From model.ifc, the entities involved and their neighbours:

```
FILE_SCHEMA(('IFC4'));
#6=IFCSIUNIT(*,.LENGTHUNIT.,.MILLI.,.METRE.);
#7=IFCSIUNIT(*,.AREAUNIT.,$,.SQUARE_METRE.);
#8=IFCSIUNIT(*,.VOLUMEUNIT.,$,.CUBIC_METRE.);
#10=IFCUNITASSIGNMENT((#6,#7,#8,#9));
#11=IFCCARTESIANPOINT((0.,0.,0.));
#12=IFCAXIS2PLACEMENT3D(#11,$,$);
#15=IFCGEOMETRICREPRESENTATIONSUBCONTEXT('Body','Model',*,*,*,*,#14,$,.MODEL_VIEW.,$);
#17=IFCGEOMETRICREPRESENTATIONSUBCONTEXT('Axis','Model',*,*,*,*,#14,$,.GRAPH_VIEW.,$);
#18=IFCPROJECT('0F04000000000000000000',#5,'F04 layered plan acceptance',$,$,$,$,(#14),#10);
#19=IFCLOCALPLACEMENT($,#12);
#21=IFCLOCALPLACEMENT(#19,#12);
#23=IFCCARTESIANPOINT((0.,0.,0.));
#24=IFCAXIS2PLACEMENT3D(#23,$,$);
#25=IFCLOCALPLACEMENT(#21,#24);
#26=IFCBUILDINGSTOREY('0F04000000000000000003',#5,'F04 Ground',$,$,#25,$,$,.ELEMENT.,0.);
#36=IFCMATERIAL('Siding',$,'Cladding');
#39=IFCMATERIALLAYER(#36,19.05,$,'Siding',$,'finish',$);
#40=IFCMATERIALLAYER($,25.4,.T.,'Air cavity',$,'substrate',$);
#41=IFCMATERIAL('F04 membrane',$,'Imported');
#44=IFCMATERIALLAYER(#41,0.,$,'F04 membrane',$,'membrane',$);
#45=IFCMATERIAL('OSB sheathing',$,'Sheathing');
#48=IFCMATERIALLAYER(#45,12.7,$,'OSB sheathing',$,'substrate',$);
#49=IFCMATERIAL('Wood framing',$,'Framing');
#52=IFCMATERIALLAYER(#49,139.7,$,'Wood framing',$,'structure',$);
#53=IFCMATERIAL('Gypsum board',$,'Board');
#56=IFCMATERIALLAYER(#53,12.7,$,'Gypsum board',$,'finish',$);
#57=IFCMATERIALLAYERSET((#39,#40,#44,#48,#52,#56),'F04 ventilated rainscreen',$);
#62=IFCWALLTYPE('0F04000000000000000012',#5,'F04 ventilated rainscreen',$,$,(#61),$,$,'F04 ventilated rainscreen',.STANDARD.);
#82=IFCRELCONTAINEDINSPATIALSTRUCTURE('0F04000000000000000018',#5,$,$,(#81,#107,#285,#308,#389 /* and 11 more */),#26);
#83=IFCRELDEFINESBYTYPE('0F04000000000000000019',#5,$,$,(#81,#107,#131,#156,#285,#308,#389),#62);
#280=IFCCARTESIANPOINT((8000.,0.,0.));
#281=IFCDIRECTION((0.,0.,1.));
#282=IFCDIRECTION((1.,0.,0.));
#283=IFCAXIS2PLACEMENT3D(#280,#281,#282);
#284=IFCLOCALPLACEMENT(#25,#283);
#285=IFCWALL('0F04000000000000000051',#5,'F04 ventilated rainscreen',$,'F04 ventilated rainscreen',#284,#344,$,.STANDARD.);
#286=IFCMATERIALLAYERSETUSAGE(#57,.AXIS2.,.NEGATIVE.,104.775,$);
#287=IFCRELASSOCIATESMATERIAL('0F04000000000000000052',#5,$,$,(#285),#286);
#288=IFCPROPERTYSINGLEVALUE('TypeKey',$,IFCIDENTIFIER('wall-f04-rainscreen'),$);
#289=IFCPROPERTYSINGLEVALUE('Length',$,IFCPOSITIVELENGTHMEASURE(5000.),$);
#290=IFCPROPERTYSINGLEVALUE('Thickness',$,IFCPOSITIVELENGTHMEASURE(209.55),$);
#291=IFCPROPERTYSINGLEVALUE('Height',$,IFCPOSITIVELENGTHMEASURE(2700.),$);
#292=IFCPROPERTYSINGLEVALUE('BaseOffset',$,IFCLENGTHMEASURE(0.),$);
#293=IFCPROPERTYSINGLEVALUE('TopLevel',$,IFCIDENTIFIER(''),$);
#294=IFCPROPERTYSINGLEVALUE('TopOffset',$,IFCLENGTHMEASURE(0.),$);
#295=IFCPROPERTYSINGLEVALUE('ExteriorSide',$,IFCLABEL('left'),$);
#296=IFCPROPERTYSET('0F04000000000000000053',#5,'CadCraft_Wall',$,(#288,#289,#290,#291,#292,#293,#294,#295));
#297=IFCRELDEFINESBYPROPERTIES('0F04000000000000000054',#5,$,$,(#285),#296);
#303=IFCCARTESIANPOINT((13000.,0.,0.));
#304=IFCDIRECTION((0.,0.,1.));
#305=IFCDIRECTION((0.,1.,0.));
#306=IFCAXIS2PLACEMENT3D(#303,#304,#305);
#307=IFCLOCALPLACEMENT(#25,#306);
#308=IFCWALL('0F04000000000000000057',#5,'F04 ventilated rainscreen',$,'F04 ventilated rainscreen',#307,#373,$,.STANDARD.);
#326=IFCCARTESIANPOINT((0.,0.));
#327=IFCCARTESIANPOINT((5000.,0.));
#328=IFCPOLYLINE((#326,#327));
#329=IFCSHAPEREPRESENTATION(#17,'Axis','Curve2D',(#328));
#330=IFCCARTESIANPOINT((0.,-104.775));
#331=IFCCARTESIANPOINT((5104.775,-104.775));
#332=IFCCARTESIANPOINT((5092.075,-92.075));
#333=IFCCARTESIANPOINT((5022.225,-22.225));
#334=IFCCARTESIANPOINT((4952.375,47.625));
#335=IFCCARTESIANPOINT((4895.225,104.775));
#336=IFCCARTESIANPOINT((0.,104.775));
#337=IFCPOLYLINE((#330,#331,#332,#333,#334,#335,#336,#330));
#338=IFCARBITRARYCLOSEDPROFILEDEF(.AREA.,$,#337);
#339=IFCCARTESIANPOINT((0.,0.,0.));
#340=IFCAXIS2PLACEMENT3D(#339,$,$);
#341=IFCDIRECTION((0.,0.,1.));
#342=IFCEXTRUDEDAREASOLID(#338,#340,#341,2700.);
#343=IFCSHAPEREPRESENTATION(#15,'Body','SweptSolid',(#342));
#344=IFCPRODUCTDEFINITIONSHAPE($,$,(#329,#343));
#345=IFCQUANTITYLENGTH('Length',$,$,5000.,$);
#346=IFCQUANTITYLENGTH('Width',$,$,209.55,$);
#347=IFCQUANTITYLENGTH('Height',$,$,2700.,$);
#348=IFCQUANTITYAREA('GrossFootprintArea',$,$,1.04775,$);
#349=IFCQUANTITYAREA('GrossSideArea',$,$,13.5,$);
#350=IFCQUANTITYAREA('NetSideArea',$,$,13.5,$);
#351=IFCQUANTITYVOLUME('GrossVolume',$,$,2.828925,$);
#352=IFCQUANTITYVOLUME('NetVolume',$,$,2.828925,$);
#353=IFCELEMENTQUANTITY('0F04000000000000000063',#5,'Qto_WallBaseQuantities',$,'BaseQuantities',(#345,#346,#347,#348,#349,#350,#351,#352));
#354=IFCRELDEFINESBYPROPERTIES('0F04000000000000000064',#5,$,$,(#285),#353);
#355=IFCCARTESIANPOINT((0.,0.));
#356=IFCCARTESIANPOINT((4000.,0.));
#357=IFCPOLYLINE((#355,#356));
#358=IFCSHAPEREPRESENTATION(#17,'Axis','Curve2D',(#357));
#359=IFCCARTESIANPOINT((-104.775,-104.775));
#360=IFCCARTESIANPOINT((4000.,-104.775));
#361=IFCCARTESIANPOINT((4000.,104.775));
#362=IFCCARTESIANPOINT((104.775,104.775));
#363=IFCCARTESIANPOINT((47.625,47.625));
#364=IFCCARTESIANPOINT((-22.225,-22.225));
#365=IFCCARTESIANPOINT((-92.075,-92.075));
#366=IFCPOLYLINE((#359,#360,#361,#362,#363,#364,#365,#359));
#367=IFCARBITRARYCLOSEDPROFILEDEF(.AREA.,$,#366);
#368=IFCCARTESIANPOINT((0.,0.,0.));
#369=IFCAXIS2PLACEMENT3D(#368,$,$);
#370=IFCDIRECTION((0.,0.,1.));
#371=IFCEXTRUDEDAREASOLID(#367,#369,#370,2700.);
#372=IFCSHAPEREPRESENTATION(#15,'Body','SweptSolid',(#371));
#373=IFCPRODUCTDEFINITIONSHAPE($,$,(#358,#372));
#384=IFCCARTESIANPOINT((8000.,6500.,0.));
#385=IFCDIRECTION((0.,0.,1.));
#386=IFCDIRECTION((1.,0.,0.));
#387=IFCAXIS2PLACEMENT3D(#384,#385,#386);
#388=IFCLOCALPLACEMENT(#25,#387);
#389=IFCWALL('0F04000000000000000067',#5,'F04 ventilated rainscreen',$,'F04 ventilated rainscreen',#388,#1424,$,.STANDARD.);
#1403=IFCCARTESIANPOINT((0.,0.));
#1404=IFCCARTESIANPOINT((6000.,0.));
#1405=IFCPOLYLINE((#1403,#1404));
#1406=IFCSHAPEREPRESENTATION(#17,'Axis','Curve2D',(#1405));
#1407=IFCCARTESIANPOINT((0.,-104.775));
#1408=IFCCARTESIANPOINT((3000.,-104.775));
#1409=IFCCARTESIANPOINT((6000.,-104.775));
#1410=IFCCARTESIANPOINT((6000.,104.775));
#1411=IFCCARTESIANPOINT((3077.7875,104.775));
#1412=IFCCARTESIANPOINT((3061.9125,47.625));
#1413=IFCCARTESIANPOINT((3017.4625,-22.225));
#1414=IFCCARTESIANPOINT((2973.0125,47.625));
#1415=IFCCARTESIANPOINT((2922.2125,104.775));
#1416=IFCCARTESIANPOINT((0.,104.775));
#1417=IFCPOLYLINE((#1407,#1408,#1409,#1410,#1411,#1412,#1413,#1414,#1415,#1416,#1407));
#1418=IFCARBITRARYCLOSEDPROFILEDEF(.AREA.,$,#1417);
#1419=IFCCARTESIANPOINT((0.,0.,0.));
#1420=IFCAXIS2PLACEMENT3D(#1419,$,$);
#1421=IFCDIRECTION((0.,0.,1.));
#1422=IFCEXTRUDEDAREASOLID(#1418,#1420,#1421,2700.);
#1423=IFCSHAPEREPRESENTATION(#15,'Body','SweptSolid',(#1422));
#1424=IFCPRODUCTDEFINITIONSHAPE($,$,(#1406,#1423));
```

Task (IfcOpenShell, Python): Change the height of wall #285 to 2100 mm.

```python
import ifcopenshell
import ifcopenshell.api.pset
import ifcopenshell.geom
import ifcopenshell.util.element
import ifcopenshell.util.representation
import ifcopenshell.util.shape
import ifcopenshell.util.unit

model = ifcopenshell.open("model.ifc")
unit_scale = ifcopenshell.util.unit.calculate_unit_scale(model)
area_scale = ifcopenshell.util.unit.calculate_unit_scale(model, "AREAUNIT")
volume_scale = ifcopenshell.util.unit.calculate_unit_scale(model, "VOLUMEUNIT")
settings = ifcopenshell.geom.settings()


def volume(element):
    """Net volume in cubic metres, openings subtracted."""
    shape = ifcopenshell.geom.create_shape(settings, element)
    return ifcopenshell.util.shape.get_volume(shape.geometry)


wall = model.by_guid("0F04000000000000000051")
before = volume(wall)

body = ifcopenshell.util.representation.get_representation(wall, "Model", "Body")
solid = body.Items[0]
old_height = solid.Depth
solid.Depth = 2100.0
after = volume(wall)
thickness = 0.2096  # wall thickness in metres

# Update the stored height, areas and volumes.
pset = model.by_id(ifcopenshell.util.element.get_pset(wall, "CadCraft_Wall", should_inherit=False)["id"])
ifcopenshell.api.pset.edit_pset(model, pset=pset, properties={
    "Height": model.create_entity("IfcPositiveLengthMeasure", solid.Depth),
})
qto = model.by_id(ifcopenshell.util.element.get_pset(wall, "Qto_WallBaseQuantities", should_inherit=False)["id"])
ifcopenshell.api.pset.edit_qto(model, qto=qto, properties={
    "Height": solid.Depth,
    "GrossSideArea": ifcopenshell.util.element.get_pset(wall, "Qto_WallBaseQuantities", "GrossSideArea") * solid.Depth / old_height,
    "NetSideArea": after / thickness / area_scale,
    "GrossVolume": ifcopenshell.util.element.get_pset(wall, "Qto_WallBaseQuantities", "GrossVolume") * solid.Depth / old_height,
    "NetVolume": after / volume_scale,
})

print(f"height {old_height:g} -> {solid.Depth:g}, volume {before:.3f} -> {after:.3f} m3")

model.write("model_rev.ifc")
```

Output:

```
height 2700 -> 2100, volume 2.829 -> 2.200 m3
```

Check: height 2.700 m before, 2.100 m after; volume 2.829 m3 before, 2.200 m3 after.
